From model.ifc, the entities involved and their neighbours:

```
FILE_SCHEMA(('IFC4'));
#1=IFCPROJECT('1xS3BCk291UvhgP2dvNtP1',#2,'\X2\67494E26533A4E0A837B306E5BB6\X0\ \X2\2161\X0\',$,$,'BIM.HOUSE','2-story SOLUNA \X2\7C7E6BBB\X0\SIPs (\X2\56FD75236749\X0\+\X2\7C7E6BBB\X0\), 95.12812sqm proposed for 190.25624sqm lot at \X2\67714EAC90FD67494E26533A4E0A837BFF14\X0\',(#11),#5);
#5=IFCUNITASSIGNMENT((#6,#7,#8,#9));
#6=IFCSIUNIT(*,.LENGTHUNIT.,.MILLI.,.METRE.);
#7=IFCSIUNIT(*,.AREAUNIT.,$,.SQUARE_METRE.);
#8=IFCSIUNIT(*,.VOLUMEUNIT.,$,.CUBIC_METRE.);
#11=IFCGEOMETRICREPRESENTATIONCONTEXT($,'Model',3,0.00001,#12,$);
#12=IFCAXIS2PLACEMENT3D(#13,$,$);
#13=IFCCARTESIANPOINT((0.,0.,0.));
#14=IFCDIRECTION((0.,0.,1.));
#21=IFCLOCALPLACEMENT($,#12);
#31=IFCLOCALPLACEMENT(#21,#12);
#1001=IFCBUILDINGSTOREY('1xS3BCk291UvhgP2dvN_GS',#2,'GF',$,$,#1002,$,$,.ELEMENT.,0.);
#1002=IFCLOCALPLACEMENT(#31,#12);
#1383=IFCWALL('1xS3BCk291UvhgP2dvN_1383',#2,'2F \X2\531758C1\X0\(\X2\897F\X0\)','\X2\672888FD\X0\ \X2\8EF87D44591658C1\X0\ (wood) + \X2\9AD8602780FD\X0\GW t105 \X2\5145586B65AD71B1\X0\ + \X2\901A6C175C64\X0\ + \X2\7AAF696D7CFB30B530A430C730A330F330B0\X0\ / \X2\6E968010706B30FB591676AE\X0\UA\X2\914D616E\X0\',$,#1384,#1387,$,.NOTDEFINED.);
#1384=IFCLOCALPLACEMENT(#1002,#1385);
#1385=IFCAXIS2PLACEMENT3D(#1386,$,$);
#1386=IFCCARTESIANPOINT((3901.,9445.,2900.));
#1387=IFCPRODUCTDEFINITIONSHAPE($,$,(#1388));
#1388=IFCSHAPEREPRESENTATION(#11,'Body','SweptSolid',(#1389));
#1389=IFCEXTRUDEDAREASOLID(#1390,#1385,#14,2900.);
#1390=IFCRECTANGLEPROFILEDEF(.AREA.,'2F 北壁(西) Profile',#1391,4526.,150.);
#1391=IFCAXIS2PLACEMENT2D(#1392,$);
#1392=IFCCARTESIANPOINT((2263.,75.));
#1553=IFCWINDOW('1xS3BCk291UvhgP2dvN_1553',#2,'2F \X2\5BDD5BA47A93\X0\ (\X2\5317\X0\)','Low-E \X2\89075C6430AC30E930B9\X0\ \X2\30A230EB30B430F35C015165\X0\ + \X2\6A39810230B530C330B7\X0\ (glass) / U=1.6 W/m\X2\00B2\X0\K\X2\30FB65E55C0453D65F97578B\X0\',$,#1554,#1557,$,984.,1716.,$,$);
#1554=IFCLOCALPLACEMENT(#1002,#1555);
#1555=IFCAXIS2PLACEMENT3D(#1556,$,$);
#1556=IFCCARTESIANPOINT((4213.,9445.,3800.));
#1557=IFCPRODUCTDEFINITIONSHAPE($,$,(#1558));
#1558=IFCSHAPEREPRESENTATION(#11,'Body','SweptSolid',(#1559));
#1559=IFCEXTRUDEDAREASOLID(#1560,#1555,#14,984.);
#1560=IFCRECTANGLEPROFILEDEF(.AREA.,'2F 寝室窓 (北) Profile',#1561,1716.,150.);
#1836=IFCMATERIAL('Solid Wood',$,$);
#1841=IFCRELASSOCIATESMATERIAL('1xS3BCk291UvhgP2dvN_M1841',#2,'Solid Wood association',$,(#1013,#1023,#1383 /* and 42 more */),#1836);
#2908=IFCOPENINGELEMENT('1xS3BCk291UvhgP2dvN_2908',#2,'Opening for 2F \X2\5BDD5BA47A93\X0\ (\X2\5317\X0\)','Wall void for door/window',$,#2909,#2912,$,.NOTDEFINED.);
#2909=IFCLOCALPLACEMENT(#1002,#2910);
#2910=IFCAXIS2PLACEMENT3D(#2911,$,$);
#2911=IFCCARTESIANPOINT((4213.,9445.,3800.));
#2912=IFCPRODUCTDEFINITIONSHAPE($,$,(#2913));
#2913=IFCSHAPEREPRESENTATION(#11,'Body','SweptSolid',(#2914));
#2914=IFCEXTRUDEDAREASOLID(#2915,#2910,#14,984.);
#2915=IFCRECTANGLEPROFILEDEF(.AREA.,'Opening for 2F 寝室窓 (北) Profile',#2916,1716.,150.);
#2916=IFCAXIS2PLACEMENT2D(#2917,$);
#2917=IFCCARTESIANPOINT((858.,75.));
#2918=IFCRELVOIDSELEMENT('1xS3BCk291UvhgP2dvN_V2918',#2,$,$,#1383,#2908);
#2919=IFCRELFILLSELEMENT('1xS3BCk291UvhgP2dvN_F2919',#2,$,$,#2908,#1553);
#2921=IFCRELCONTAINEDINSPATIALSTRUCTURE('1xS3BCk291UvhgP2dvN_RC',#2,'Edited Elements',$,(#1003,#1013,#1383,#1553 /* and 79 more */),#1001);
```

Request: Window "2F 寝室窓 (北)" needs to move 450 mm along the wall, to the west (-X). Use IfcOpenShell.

```python
import ifcopenshell
import ifcopenshell.api.geometry
import ifcopenshell.util.placement
import ifcopenshell.util.unit

model = ifcopenshell.open("model.ifc")
unit_scale = ifcopenshell.util.unit.calculate_unit_scale(model)

window = model.by_guid("1xS3BCk291UvhgP2dvN_1553")
opening = window.FillsVoids[0].RelatingOpeningElement
wall = opening.VoidsElements[0].RelatingBuildingElement

wall_matrix = ifcopenshell.util.placement.get_local_placement(wall.ObjectPlacement)
shift = wall_matrix[:3, 0] * -0.45 / unit_scale
before = ifcopenshell.util.placement.get_local_placement(window.ObjectPlacement)[:3, 3].copy()

# The window is not placed relative to its opening, so move both.
for product in (opening, window):
    matrix = ifcopenshell.util.placement.get_local_placement(product.ObjectPlacement)
    matrix[:3, 3] += shift
    ifcopenshell.api.geometry.edit_object_placement(model, product=product, matrix=matrix, is_si=False)

after = ifcopenshell.util.placement.get_local_placement(window.ObjectPlacement)[:3, 3]
print("window moved by", (after - before).round(3) + 0.0)

model.write("model_rev.ifc")
```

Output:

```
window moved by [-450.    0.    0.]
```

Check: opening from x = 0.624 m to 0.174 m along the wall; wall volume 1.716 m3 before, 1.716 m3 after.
